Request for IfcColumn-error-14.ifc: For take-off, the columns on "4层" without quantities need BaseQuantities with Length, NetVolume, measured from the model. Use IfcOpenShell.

First a look at what the model holds.

```python
import ifcopenshell
import ifcopenshell.util.element
import ifcopenshell.util.unit

model = ifcopenshell.open("IfcColumn-error-14.ifc")
print(model.schema)
for unit_type in ("LENGTHUNIT", "AREAUNIT", "VOLUMEUNIT"):
    print(unit_type, ifcopenshell.util.unit.calculate_unit_scale(model, unit_type))
storey = next(s for s in model.by_type("IfcBuildingStorey") if s.Name == "4层")
columns = [e for e in ifcopenshell.util.element.get_decomposition(storey) if e.is_a("IfcColumn")]
for e in sorted(columns, key=lambda e: e.id()):
    print(e.id(), e.is_a(), e.Name, list(ifcopenshell.util.element.get_psets(e, qtos_only=True)), sep=" | ")
```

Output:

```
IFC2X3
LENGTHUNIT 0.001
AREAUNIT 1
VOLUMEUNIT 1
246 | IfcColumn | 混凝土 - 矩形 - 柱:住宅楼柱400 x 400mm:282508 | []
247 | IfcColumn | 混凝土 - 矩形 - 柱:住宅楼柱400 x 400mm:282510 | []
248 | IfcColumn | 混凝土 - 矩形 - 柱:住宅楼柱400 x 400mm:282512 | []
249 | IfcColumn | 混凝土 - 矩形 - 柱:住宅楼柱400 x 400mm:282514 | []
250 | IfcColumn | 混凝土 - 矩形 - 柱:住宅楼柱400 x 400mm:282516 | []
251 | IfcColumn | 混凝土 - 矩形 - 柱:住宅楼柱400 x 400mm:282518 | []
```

```python
import ifcopenshell
import ifcopenshell.api.pset
import ifcopenshell.geom
import ifcopenshell.util.element
import ifcopenshell.util.shape
import ifcopenshell.util.unit

model = ifcopenshell.open("IfcColumn-error-14.ifc")
unit_scale = ifcopenshell.util.unit.calculate_unit_scale(model)
volume_scale = ifcopenshell.util.unit.calculate_unit_scale(model, "VOLUMEUNIT")
settings = ifcopenshell.geom.settings()

storey = next(s for s in model.by_type("IfcBuildingStorey") if s.Name == "4层")
columns = [e for e in ifcopenshell.util.element.get_decomposition(storey) if e.is_a("IfcColumn")]

for e in sorted(columns, key=lambda e: e.id()):
    if ifcopenshell.util.element.get_psets(e, qtos_only=True, should_inherit=False):
        continue
    # Geometry comes back in metres, in the element's own axes.
    shape = ifcopenshell.geom.create_shape(settings, e)
    values = {
        "Length": ifcopenshell.util.shape.get_z(shape.geometry) / unit_scale,
        "NetVolume": ifcopenshell.util.shape.get_volume(shape.geometry) / volume_scale,
    }
    qto = ifcopenshell.api.pset.add_qto(model, product=e, name="BaseQuantities")
    ifcopenshell.api.pset.edit_qto(model, qto=qto, properties=values)
    print(e.id(), {k: round(v, 3) for k, v in values.items()})

model.write("IfcColumn-error-14_edited.ifc")
```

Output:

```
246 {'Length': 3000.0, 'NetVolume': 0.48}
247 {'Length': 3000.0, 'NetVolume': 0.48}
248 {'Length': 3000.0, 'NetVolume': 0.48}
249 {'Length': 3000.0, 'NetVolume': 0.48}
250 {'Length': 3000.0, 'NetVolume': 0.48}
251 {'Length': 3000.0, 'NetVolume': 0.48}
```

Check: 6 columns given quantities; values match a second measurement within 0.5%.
